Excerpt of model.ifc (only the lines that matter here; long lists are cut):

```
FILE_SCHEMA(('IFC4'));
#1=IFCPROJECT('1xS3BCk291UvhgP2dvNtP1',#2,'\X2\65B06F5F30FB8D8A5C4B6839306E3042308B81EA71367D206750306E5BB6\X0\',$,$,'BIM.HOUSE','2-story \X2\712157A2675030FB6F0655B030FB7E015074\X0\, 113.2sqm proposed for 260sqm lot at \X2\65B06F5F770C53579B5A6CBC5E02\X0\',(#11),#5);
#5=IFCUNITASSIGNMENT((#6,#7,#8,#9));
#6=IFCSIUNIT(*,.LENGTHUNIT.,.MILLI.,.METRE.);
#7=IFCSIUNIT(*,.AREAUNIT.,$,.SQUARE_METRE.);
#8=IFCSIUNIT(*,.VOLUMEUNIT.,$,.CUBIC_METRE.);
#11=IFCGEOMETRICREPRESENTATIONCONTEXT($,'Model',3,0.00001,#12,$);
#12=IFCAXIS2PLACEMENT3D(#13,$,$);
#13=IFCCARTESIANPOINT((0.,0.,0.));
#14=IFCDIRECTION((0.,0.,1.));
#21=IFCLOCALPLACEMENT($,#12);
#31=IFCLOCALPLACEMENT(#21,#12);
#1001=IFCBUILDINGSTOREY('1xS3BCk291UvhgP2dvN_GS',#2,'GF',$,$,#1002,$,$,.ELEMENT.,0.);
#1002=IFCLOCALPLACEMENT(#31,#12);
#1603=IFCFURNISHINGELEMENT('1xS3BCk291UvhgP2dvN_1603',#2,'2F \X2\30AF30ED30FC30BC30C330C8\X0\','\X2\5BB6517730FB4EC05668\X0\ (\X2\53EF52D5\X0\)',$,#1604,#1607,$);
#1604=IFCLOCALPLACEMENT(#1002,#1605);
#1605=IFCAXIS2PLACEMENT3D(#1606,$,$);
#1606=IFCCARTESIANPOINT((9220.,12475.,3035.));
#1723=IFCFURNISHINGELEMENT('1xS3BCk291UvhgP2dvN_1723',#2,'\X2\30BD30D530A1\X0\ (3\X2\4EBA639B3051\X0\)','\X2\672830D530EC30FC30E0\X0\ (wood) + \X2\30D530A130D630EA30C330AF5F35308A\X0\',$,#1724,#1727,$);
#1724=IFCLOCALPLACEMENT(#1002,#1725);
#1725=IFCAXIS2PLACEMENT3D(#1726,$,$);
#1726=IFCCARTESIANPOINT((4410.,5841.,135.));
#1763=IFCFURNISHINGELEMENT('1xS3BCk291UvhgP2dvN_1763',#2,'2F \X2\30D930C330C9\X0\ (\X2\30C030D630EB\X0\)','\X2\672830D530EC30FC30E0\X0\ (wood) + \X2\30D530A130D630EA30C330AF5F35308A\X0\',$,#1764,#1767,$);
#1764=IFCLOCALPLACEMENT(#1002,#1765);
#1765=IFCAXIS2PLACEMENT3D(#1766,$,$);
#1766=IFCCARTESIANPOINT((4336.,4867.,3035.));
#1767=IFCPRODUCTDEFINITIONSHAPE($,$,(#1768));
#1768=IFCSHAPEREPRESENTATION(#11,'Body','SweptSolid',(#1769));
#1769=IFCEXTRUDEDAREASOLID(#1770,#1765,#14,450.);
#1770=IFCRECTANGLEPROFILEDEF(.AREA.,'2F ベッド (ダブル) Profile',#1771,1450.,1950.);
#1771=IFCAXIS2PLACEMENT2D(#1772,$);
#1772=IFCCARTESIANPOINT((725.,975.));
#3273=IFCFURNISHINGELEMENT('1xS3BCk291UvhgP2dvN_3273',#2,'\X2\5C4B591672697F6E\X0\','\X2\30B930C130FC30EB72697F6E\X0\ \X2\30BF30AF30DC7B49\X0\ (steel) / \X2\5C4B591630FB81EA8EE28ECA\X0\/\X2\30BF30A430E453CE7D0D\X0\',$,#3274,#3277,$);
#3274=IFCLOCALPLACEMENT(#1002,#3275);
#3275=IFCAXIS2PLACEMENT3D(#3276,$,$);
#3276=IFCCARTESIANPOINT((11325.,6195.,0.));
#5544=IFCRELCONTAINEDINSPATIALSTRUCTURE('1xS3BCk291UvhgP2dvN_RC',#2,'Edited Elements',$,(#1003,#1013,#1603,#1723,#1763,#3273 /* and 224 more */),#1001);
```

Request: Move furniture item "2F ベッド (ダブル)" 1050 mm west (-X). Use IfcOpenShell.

```python
import ifcopenshell
import ifcopenshell.api.geometry
import ifcopenshell.util.placement

model = ifcopenshell.open("model.ifc")

item = model.by_id(1763)
matrix = ifcopenshell.util.placement.get_local_placement(item.ObjectPlacement)
matrix[0, 3] -= 1050.0
ifcopenshell.api.geometry.edit_object_placement(model, product=item, matrix=matrix, is_si=False)

print(ifcopenshell.util.placement.get_local_placement(item.ObjectPlacement).round(3) + 0.0)

model.write("model_rev.ifc")
```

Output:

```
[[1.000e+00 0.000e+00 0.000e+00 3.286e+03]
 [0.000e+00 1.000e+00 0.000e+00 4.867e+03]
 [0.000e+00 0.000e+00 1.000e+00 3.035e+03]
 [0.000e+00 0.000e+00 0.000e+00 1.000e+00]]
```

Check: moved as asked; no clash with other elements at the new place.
